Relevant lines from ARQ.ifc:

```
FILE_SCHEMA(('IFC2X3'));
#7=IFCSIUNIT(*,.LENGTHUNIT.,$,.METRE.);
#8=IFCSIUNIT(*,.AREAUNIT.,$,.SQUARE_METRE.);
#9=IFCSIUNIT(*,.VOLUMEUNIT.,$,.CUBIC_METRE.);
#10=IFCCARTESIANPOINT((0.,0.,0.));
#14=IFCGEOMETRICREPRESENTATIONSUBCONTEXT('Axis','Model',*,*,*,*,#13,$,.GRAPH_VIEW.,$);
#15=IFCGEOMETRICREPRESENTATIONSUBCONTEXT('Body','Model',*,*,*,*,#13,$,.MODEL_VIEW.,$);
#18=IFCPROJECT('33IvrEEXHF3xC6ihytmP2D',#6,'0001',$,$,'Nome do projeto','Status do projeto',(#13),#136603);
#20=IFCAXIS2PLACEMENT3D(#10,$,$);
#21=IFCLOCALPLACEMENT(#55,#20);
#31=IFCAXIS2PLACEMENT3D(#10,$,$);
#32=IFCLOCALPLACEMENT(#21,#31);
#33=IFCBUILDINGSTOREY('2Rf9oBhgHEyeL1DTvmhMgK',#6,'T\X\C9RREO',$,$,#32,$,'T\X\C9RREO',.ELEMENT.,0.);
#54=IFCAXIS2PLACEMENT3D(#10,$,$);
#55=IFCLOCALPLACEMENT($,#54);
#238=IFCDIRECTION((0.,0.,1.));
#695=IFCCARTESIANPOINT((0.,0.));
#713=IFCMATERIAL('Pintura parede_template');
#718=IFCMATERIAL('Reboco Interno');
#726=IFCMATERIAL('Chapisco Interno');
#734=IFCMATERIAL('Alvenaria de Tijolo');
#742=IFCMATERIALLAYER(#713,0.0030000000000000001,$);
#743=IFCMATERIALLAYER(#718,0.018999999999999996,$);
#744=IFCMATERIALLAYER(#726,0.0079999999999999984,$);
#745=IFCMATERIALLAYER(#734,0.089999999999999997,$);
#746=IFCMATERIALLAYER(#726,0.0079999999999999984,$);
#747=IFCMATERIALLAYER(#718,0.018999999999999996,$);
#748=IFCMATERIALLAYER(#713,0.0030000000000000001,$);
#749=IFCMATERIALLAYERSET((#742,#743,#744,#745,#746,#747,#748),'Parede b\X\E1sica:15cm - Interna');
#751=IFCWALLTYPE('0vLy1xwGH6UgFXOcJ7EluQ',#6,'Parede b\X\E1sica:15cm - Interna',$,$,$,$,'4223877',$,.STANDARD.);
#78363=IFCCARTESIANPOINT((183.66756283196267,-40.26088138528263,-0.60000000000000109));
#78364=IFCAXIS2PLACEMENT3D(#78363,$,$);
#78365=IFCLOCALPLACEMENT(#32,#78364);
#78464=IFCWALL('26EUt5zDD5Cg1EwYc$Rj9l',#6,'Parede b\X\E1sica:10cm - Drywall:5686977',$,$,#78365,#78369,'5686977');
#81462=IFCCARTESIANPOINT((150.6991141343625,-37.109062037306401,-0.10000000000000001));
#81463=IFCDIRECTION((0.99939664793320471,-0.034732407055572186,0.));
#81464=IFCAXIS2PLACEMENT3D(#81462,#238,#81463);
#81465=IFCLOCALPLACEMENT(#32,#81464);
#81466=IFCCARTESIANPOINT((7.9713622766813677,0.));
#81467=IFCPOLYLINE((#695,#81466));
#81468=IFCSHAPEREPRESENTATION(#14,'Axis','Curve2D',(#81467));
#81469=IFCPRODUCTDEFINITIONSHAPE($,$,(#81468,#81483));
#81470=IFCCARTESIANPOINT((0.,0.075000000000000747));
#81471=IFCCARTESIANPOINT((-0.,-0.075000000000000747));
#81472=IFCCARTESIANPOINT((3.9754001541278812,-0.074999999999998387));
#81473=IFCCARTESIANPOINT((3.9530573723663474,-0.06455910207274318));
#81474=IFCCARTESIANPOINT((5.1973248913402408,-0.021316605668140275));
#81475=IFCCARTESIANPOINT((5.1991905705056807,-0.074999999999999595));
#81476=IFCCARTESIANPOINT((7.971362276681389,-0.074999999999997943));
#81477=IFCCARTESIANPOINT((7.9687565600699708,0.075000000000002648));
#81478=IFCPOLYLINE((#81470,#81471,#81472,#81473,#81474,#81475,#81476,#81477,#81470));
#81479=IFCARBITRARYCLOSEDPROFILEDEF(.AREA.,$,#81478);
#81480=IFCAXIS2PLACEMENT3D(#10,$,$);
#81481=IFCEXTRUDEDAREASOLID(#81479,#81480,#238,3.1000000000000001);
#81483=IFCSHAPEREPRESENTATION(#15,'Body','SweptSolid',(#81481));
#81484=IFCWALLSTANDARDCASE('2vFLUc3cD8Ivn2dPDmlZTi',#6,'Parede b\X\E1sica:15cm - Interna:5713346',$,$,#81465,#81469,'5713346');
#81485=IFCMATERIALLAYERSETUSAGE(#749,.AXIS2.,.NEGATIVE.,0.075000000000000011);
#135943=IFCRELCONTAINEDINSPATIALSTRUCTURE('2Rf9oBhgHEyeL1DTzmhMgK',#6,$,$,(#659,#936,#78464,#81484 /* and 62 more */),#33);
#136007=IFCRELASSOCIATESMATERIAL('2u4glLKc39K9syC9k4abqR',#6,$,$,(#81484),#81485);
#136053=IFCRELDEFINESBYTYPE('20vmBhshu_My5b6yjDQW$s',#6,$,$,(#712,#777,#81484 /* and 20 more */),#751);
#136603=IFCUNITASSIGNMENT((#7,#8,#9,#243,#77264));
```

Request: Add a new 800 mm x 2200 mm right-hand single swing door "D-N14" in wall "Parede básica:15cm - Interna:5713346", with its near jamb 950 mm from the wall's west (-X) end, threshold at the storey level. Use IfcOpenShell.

```python
import numpy as np
import ifcopenshell
import ifcopenshell.api.feature
import ifcopenshell.api.geometry
import ifcopenshell.api.root
import ifcopenshell.api.spatial
import ifcopenshell.api.type
import ifcopenshell.geom
import ifcopenshell.util.element
import ifcopenshell.util.placement
import ifcopenshell.util.representation
import ifcopenshell.util.shape
import ifcopenshell.util.unit

model = ifcopenshell.open("ARQ.ifc")
unit_scale = ifcopenshell.util.unit.calculate_unit_scale(model)
settings = ifcopenshell.geom.settings()


def volume(element):
    """Net volume in cubic metres, openings subtracted."""
    shape = ifcopenshell.geom.create_shape(settings, element)
    return ifcopenshell.util.shape.get_volume(shape.geometry)


wall = model.by_guid("2vFLUc3cD8Ivn2dPDmlZTi")
storey = ifcopenshell.util.element.get_container(wall, ifc_class="IfcBuildingStorey")
context = ifcopenshell.util.representation.get_context(model, "Model", "Body", "MODEL_VIEW")
before = volume(wall)

width, height, from_end, sill = 0.8, 2.2, 0.95, 0.0  # metres

# The wall runs along its own X axis, and the end named is its -X end.
wall_shape = ifcopenshell.geom.create_shape(settings, wall)
x, y, z = ifcopenshell.util.shape.get_vertices(wall_shape.geometry).T
start = x.min() + from_end
face, thickness = float(y.min()), float(y.max() - y.min())
wall_matrix = ifcopenshell.util.placement.get_local_placement(wall.ObjectPlacement)
level = ifcopenshell.util.placement.get_local_placement(storey.ObjectPlacement)[2, 3]


def in_wall(x, y):
    """Placement at x, y metres in the wall's axes, at sill height."""
    matrix = wall_matrix.copy()
    matrix[:, 3] = wall_matrix @ np.array([x / unit_scale, y / unit_scale, 0.0, 1.0])
    matrix[2, 3] = level + sill / unit_scale
    return matrix


# Opening: a box that overshoots both wall faces by 50 mm.
opening = ifcopenshell.api.root.create_entity(model, ifc_class="IfcOpeningElement")
box = ifcopenshell.api.geometry.add_wall_representation(
    model, context=context, length=width, height=height, thickness=thickness + 0.1
)
ifcopenshell.api.geometry.assign_representation(model, product=opening, representation=box)
ifcopenshell.api.geometry.edit_object_placement(model, product=opening, matrix=in_wall(start, face - 0.05), is_si=False)
ifcopenshell.api.feature.add_feature(model, feature=opening, element=wall)

door = ifcopenshell.api.root.create_entity(model, ifc_class="IfcDoor", name="D-N14")
door.OverallWidth, door.OverallHeight = width / unit_scale, height / unit_scale
body = ifcopenshell.api.geometry.add_door_representation(
    model,
    context=context,
    overall_width=door.OverallWidth,
    overall_height=door.OverallHeight,
    operation_type="SINGLE_SWING_RIGHT",
    lining_properties={"LiningDepth": thickness / unit_scale, "ThresholdDepth": thickness / unit_scale},
)
ifcopenshell.api.geometry.assign_representation(model, product=door, representation=body)
ifcopenshell.api.spatial.assign_container(model, products=[door], relating_structure=storey)
fills = ifcopenshell.api.feature.add_filling(model, opening=opening, element=door)
fills.OwnerHistory = door.OwnerHistory  # required in IFC2X3

# IFC2X3 keeps the operation on the door style.
style = ifcopenshell.api.root.create_entity(model, ifc_class="IfcDoorStyle", name="D-N14")
style.OperationType, style.ConstructionType = "SINGLE_SWING_RIGHT", "NOTDEFINED"
style.ParameterTakesPrecedence = style.Sizeable = False
ifcopenshell.api.type.assign_type(model, related_objects=[door], relating_type=style)

# The lining spans the wall, so the door starts at the wall face.
ifcopenshell.api.geometry.edit_object_placement(model, product=door, matrix=in_wall(start, face), is_si=False)

after = volume(wall)

print(f"wall volume {before:.3f} -> {after:.3f} m3")

model.write("ARQ-out.ifc")
```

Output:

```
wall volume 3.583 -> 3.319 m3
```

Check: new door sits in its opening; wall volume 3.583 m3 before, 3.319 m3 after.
